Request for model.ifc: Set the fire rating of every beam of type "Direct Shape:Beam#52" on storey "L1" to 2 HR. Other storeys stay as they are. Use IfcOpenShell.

First a look at what the model holds.

```python
import ifcopenshell
import ifcopenshell.util.element

model = ifcopenshell.open("model.ifc")
print(model.schema)
storey = next(s for s in model.by_type("IfcBuildingStorey") if s.Name == "L1")
beams = [e for e in ifcopenshell.util.element.get_decomposition(storey) if e.is_a("IfcBeam")]
seen = {}
for e in beams:
    element_type = ifcopenshell.util.element.get_type(e)
    key = (element_type.Name if element_type != e and element_type else None, ifcopenshell.util.element.get_pset(e, "Pset_BeamCommon", "FireRating"))
    seen[key] = seen.get(key, 0) + 1
for (name, value), count in sorted(seen.items(), key=str):
    print(count, "x", name, "|", value)
```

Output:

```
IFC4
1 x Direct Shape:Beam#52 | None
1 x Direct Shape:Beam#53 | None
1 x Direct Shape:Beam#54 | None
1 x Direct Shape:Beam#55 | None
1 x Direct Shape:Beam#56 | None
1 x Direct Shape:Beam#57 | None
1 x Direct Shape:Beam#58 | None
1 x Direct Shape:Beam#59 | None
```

```python
import ifcopenshell
import ifcopenshell.api.pset
import ifcopenshell.util.element

model = ifcopenshell.open("model.ifc")

storey = next(s for s in model.by_type("IfcBuildingStorey") if s.Name == "L1")
beams = [e for e in ifcopenshell.util.element.get_decomposition(storey) if e.is_a("IfcBeam")]

count = 0
for e in beams:
    element_type = ifcopenshell.util.element.get_type(e)
    if element_type in (None, e) or element_type.Name != "Direct Shape:Beam#52":
        continue
    # add_pset returns the element's existing set when there is one.
    pset = ifcopenshell.api.pset.add_pset(model, product=e, name="Pset_BeamCommon")
    ifcopenshell.api.pset.edit_pset(model, pset=pset, properties={"FireRating": "2 HR"})
    count += 1

print(count, "beams updated")

model.write("model_v2.ifc")
```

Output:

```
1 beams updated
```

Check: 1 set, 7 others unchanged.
